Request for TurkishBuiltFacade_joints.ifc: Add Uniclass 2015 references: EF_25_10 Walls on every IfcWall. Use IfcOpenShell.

First a look at what the model holds.

```python
import ifcopenshell

model = ifcopenshell.open("TurkishBuiltFacade_joints.ifc")
print(model.schema)
print("classifications:", [c.Name for c in model.by_type("IfcClassification")])
for ifc_class in ("IfcDoor", "IfcRoof", "IfcStair", "IfcWall", "IfcWindow"):
    print(ifc_class, len(model.by_type(ifc_class)))
```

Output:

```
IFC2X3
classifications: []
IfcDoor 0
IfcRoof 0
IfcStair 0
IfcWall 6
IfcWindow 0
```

```python
import ifcopenshell
import ifcopenshell.api.classification

model = ifcopenshell.open("TurkishBuiltFacade_joints.ifc")

# IFC2X3 requires Source and Edition and has no link from the project to the system.
system = model.create_entity("IfcClassification", Source="NBS", Edition="2015", Name="Uniclass 2015")

codes = {
    "IfcWall": ("EF_25_10", "Walls"),
}
for ifc_class, (code, name) in codes.items():
    products = model.by_type(ifc_class)
    ifcopenshell.api.classification.add_reference(
        model, products=products, classification=system, identification=code, name=name
    )
    print(code, len(products))

model.write("TurkishBuiltFacade_joints-out.ifc")
```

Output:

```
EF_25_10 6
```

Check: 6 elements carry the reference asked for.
